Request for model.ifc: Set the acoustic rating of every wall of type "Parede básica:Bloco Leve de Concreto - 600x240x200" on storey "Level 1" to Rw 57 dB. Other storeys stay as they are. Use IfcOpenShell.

First a look at what the model holds.

```python
import ifcopenshell
import ifcopenshell.util.element

model = ifcopenshell.open("model.ifc")
print(model.schema)
storey = next(s for s in model.by_type("IfcBuildingStorey") if s.Name == "Level 1")
walls = [e for e in ifcopenshell.util.element.get_decomposition(storey) if e.is_a("IfcWall")]
seen = {}
for e in walls:
    element_type = ifcopenshell.util.element.get_type(e)
    key = (element_type.Name if element_type != e and element_type else None, ifcopenshell.util.element.get_pset(e, "Pset_WallCommon", "AcousticRating"))
    seen[key] = seen.get(key, 0) + 1
for (name, value), count in sorted(seen.items(), key=str):
    print(count, "x", name, "|", value)
```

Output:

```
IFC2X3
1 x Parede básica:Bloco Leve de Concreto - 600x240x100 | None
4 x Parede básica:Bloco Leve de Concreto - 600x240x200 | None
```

```python
import ifcopenshell
import ifcopenshell.api.pset
import ifcopenshell.util.element

model = ifcopenshell.open("model.ifc")

storey = next(s for s in model.by_type("IfcBuildingStorey") if s.Name == "Level 1")
walls = [e for e in ifcopenshell.util.element.get_decomposition(storey) if e.is_a("IfcWall")]

count = 0
for e in walls:
    element_type = ifcopenshell.util.element.get_type(e)
    if element_type in (None, e) or element_type.Name != "Parede básica:Bloco Leve de Concreto - 600x240x200":
        continue
    # add_pset returns the element's existing set when there is one.
    pset = ifcopenshell.api.pset.add_pset(model, product=e, name="Pset_WallCommon")
    ifcopenshell.api.pset.edit_pset(model, pset=pset, properties={"AcousticRating": "Rw 57 dB"})
    count += 1

print(count, "walls updated")

model.write("model_edited.ifc")
```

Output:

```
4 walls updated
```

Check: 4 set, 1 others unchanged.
